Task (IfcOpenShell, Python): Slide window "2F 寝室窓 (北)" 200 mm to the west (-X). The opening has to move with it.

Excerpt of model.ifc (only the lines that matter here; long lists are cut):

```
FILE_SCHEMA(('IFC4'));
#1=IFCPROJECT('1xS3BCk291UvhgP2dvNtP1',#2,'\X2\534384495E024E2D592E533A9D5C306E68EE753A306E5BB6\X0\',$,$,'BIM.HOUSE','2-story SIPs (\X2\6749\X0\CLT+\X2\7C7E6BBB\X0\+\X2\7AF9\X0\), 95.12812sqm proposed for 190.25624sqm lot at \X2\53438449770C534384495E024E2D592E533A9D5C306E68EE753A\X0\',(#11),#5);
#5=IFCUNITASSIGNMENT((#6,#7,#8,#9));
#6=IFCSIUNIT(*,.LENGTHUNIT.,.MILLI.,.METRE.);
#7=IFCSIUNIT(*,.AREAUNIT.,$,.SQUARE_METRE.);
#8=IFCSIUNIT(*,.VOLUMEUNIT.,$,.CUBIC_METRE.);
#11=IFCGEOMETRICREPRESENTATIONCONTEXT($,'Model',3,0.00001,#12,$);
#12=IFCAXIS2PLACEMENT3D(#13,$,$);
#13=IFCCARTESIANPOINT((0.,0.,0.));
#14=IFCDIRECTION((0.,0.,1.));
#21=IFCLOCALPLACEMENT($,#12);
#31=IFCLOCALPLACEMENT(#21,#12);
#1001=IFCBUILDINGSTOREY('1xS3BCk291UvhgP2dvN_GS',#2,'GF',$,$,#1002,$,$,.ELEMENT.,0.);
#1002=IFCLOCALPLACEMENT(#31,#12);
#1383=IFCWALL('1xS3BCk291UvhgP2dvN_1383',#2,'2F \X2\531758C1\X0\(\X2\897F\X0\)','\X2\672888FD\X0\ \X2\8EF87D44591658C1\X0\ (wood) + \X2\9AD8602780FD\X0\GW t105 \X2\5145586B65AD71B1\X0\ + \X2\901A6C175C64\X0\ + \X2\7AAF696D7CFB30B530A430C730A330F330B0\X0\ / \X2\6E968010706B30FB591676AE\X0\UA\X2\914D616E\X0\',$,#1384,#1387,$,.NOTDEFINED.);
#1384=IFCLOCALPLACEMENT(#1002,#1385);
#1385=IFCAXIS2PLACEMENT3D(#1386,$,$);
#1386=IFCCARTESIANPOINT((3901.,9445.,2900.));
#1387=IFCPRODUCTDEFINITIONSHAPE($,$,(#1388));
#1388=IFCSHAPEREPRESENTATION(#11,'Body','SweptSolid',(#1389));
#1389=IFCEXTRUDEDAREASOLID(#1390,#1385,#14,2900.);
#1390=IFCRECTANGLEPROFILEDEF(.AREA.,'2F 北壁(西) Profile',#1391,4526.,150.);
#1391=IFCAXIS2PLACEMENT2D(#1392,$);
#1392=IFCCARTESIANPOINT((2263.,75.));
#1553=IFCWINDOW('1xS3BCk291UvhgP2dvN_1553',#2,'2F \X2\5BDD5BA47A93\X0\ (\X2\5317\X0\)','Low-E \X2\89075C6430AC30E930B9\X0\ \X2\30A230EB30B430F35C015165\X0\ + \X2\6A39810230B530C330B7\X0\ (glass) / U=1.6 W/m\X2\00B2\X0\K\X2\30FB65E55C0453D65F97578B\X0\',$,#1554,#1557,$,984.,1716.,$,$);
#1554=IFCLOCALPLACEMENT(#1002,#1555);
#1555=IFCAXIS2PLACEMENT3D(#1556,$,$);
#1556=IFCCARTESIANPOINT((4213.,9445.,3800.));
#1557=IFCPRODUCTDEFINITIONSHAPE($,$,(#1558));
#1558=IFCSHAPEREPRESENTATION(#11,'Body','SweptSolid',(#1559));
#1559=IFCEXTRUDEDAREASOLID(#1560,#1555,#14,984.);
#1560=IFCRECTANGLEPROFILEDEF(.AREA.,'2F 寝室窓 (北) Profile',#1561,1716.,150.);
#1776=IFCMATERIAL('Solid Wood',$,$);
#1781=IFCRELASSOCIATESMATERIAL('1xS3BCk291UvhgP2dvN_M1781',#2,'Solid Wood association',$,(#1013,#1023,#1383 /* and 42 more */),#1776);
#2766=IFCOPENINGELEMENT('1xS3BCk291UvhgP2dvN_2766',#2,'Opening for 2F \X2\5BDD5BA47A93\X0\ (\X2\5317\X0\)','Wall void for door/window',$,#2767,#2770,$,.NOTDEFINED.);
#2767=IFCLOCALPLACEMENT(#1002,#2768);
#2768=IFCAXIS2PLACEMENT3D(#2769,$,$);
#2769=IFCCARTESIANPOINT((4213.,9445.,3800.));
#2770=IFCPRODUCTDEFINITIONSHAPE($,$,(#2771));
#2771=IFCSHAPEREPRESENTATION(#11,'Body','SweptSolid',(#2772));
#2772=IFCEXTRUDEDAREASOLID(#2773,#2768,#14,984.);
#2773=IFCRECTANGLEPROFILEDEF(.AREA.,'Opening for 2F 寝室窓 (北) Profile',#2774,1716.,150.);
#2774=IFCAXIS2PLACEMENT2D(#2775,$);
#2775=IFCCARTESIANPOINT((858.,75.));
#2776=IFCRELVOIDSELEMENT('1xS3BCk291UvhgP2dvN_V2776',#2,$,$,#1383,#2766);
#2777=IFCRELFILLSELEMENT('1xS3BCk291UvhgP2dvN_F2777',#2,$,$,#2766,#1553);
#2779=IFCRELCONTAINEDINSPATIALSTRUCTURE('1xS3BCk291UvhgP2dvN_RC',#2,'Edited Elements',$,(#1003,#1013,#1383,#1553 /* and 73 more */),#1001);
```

```python
import ifcopenshell
import ifcopenshell.api.geometry
import ifcopenshell.util.placement
import ifcopenshell.util.unit

model = ifcopenshell.open("model.ifc")
unit_scale = ifcopenshell.util.unit.calculate_unit_scale(model)

window = model.by_id(1553)
opening = window.FillsVoids[0].RelatingOpeningElement
wall = opening.VoidsElements[0].RelatingBuildingElement

wall_matrix = ifcopenshell.util.placement.get_local_placement(wall.ObjectPlacement)
shift = wall_matrix[:3, 0] * -0.2 / unit_scale
before = ifcopenshell.util.placement.get_local_placement(window.ObjectPlacement)[:3, 3].copy()

# The window is not placed relative to its opening, so move both.
for product in (opening, window):
    matrix = ifcopenshell.util.placement.get_local_placement(product.ObjectPlacement)
    matrix[:3, 3] += shift
    ifcopenshell.api.geometry.edit_object_placement(model, product=product, matrix=matrix, is_si=False)

after = ifcopenshell.util.placement.get_local_placement(window.ObjectPlacement)[:3, 3]
print("window moved by", (after - before).round(3) + 0.0)

model.write("model_edited.ifc")
```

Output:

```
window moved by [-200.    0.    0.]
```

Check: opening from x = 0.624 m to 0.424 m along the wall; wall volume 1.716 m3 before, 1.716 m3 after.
